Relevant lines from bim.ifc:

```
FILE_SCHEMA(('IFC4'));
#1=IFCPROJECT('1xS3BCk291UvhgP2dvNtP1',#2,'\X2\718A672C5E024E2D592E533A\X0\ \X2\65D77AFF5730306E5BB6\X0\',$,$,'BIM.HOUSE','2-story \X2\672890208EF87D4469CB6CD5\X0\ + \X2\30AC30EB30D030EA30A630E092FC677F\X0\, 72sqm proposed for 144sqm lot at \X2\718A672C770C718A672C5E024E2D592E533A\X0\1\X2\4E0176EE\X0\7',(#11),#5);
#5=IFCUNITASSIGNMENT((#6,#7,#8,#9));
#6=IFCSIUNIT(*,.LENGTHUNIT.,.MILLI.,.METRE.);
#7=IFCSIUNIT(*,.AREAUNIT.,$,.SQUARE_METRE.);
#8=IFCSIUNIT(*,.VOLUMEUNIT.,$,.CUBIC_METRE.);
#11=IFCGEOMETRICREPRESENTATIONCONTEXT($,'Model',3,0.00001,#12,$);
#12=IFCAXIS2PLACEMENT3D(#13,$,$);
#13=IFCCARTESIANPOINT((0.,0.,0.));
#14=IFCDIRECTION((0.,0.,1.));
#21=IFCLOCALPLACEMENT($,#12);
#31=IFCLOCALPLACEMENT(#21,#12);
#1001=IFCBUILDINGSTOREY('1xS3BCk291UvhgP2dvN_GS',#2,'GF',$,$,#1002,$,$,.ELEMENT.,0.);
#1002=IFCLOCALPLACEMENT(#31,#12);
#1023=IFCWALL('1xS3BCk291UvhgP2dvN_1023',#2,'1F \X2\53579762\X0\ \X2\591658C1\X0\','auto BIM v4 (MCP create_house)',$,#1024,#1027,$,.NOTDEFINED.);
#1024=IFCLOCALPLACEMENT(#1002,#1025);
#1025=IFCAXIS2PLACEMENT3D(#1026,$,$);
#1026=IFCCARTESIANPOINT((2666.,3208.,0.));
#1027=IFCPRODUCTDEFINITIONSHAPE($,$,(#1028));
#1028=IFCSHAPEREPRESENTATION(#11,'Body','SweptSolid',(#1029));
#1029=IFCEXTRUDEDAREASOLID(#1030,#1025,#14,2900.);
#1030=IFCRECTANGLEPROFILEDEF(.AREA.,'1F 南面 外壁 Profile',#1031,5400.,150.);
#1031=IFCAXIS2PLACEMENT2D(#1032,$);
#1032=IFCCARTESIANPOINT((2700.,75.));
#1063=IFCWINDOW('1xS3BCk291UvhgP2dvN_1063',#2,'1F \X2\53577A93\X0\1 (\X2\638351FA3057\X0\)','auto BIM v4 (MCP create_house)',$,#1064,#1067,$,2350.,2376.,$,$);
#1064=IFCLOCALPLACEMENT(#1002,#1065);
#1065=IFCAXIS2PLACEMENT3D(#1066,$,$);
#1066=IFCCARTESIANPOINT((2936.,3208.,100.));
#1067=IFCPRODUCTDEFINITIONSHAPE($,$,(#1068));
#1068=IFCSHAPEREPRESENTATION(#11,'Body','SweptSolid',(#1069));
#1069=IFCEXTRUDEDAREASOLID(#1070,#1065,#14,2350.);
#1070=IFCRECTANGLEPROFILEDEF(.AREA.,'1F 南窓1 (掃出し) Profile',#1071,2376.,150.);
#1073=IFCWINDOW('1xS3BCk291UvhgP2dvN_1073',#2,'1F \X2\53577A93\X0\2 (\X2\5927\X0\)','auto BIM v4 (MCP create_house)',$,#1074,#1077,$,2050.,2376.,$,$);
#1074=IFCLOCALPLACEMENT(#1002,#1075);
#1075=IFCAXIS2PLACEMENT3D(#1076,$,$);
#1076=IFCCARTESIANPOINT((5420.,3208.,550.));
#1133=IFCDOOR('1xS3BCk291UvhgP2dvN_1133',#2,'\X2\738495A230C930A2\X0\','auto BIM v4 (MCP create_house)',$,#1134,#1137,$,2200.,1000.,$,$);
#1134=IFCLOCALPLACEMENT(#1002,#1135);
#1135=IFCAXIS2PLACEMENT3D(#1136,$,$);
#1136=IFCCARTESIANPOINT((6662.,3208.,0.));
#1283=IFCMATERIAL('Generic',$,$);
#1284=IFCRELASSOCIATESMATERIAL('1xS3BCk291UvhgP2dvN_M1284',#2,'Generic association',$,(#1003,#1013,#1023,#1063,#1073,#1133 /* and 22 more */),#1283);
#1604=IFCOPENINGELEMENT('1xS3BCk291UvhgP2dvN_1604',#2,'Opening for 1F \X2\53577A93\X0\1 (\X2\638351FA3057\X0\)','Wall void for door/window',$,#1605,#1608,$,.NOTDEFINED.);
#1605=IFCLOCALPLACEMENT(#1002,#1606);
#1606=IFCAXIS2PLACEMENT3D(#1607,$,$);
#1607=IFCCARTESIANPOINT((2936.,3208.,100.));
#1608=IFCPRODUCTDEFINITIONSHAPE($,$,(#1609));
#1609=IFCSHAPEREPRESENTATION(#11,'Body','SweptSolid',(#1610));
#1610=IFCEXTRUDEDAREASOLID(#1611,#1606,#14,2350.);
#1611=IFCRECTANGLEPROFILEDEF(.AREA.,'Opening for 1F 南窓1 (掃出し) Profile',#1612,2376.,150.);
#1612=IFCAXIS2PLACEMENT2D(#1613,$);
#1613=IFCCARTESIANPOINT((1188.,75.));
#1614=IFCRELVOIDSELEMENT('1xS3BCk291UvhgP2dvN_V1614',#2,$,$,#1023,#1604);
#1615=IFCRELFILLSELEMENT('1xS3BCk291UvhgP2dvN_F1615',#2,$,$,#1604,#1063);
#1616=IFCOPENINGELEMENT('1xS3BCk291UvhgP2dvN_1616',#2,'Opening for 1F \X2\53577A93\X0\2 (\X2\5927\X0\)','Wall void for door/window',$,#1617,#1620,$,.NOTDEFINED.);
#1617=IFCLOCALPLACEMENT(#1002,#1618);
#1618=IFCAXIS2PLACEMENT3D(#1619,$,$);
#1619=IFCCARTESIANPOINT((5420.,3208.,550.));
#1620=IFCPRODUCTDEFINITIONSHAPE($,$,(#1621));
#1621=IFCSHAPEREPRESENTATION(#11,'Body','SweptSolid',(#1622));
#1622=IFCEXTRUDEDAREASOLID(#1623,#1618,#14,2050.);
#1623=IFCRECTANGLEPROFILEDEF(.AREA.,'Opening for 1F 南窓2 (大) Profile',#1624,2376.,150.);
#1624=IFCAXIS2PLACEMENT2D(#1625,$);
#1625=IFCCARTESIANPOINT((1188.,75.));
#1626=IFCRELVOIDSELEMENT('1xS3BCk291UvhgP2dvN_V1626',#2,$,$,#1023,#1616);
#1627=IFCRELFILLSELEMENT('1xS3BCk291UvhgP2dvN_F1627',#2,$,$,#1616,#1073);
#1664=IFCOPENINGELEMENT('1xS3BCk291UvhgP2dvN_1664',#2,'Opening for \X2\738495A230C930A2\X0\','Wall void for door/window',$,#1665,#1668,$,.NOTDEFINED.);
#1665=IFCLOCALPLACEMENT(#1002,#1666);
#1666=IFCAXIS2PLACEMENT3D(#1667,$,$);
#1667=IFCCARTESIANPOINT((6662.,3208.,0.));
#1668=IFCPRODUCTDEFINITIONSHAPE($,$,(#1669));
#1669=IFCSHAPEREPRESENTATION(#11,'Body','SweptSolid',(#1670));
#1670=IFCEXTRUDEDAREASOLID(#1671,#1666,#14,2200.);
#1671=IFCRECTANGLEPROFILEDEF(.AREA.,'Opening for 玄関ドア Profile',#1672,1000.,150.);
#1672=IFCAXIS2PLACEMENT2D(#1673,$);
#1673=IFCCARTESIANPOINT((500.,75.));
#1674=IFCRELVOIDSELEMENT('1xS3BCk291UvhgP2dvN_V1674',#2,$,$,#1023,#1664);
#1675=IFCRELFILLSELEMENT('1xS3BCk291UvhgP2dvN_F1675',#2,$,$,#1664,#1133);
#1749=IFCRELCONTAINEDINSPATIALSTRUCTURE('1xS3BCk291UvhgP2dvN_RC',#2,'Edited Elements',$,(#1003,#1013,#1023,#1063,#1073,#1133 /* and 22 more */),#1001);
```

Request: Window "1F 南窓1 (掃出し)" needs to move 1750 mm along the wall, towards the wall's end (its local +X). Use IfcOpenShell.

```python
import ifcopenshell
import ifcopenshell.api.geometry
import ifcopenshell.util.placement
import ifcopenshell.util.unit

model = ifcopenshell.open("bim.ifc")
unit_scale = ifcopenshell.util.unit.calculate_unit_scale(model)

window = model.by_id(1063)
opening = window.FillsVoids[0].RelatingOpeningElement
wall = opening.VoidsElements[0].RelatingBuildingElement

wall_matrix = ifcopenshell.util.placement.get_local_placement(wall.ObjectPlacement)
shift = wall_matrix[:3, 0] * 1.75 / unit_scale
before = ifcopenshell.util.placement.get_local_placement(window.ObjectPlacement)[:3, 3].copy()

# The window is not placed relative to its opening, so move both.
for product in (opening, window):
    matrix = ifcopenshell.util.placement.get_local_placement(product.ObjectPlacement)
    matrix[:3, 3] += shift
    ifcopenshell.api.geometry.edit_object_placement(model, product=product, matrix=matrix, is_si=False)

after = ifcopenshell.util.placement.get_local_placement(window.ObjectPlacement)[:3, 3]
print("window moved by", (after - before).round(3) + 0.0)

model.write("bim_rev.ifc")
```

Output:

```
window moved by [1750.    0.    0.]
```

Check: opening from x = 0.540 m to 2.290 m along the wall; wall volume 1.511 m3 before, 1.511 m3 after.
